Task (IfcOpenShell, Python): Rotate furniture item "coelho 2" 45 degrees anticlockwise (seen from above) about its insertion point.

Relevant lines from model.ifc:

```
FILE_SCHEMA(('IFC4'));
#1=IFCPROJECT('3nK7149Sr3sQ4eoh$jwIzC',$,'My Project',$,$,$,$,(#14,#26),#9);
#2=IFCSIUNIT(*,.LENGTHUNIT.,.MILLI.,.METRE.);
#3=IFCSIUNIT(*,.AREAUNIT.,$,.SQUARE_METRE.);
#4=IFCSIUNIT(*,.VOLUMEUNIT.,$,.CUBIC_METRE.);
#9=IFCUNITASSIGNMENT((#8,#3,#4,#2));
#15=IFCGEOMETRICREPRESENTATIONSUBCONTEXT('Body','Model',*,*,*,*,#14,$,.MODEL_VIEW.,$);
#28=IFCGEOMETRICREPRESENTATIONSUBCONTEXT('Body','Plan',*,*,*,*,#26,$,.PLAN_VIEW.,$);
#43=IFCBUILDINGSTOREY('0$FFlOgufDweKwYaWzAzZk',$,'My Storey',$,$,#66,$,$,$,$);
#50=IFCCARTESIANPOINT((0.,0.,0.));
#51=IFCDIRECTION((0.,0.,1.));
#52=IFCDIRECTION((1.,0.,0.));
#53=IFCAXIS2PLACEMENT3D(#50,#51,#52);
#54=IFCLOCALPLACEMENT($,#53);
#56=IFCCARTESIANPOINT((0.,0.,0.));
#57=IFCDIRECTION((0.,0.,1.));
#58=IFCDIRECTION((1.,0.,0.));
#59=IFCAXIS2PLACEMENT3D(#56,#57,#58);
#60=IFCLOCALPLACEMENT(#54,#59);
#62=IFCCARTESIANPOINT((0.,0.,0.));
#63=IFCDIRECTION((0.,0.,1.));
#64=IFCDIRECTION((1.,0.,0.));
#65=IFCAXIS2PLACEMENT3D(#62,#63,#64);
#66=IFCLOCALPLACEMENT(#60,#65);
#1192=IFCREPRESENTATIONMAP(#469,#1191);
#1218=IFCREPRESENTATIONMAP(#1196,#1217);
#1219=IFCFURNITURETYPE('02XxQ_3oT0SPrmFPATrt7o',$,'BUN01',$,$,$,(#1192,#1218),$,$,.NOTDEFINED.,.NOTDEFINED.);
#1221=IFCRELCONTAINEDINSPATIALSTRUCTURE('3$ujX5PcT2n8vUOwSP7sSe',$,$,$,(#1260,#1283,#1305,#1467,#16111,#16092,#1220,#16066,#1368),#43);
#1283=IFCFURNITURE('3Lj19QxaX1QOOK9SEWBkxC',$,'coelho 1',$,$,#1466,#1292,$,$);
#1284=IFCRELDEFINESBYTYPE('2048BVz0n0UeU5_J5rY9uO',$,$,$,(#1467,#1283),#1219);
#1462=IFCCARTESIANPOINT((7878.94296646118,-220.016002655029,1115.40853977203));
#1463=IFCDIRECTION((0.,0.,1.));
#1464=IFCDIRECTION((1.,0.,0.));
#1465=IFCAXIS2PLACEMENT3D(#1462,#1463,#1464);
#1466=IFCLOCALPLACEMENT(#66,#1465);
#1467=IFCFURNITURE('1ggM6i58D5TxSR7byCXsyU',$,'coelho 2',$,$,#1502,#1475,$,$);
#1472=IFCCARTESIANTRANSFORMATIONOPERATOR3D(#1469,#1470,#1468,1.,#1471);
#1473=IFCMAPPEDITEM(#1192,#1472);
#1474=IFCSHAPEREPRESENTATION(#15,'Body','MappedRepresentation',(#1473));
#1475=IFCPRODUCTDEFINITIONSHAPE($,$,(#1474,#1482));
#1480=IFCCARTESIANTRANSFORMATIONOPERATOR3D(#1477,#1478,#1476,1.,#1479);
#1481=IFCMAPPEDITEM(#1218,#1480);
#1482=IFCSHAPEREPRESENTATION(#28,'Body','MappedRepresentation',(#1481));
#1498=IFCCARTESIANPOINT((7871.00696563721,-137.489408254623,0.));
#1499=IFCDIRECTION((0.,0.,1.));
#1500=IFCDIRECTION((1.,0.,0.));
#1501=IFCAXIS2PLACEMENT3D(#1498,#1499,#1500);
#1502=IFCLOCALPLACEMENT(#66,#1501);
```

```python
import ifcopenshell
import ifcopenshell.api.geometry
import ifcopenshell.util.placement

model = ifcopenshell.open("model.ifc")

item = model.by_guid("1ggM6i58D5TxSR7byCXsyU")
matrix = ifcopenshell.util.placement.get_local_placement(item.ObjectPlacement)
matrix = matrix @ ifcopenshell.util.placement.rotation(45, "Z")
ifcopenshell.api.geometry.edit_object_placement(model, product=item, matrix=matrix, is_si=False)

print(ifcopenshell.util.placement.get_local_placement(item.ObjectPlacement).round(3) + 0.0)

model.write("model_rev.ifc")
```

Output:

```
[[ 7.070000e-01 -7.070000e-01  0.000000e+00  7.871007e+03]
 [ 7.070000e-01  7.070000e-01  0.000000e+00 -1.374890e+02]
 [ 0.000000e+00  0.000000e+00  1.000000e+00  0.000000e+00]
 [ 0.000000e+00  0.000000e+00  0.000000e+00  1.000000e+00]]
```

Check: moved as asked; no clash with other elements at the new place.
